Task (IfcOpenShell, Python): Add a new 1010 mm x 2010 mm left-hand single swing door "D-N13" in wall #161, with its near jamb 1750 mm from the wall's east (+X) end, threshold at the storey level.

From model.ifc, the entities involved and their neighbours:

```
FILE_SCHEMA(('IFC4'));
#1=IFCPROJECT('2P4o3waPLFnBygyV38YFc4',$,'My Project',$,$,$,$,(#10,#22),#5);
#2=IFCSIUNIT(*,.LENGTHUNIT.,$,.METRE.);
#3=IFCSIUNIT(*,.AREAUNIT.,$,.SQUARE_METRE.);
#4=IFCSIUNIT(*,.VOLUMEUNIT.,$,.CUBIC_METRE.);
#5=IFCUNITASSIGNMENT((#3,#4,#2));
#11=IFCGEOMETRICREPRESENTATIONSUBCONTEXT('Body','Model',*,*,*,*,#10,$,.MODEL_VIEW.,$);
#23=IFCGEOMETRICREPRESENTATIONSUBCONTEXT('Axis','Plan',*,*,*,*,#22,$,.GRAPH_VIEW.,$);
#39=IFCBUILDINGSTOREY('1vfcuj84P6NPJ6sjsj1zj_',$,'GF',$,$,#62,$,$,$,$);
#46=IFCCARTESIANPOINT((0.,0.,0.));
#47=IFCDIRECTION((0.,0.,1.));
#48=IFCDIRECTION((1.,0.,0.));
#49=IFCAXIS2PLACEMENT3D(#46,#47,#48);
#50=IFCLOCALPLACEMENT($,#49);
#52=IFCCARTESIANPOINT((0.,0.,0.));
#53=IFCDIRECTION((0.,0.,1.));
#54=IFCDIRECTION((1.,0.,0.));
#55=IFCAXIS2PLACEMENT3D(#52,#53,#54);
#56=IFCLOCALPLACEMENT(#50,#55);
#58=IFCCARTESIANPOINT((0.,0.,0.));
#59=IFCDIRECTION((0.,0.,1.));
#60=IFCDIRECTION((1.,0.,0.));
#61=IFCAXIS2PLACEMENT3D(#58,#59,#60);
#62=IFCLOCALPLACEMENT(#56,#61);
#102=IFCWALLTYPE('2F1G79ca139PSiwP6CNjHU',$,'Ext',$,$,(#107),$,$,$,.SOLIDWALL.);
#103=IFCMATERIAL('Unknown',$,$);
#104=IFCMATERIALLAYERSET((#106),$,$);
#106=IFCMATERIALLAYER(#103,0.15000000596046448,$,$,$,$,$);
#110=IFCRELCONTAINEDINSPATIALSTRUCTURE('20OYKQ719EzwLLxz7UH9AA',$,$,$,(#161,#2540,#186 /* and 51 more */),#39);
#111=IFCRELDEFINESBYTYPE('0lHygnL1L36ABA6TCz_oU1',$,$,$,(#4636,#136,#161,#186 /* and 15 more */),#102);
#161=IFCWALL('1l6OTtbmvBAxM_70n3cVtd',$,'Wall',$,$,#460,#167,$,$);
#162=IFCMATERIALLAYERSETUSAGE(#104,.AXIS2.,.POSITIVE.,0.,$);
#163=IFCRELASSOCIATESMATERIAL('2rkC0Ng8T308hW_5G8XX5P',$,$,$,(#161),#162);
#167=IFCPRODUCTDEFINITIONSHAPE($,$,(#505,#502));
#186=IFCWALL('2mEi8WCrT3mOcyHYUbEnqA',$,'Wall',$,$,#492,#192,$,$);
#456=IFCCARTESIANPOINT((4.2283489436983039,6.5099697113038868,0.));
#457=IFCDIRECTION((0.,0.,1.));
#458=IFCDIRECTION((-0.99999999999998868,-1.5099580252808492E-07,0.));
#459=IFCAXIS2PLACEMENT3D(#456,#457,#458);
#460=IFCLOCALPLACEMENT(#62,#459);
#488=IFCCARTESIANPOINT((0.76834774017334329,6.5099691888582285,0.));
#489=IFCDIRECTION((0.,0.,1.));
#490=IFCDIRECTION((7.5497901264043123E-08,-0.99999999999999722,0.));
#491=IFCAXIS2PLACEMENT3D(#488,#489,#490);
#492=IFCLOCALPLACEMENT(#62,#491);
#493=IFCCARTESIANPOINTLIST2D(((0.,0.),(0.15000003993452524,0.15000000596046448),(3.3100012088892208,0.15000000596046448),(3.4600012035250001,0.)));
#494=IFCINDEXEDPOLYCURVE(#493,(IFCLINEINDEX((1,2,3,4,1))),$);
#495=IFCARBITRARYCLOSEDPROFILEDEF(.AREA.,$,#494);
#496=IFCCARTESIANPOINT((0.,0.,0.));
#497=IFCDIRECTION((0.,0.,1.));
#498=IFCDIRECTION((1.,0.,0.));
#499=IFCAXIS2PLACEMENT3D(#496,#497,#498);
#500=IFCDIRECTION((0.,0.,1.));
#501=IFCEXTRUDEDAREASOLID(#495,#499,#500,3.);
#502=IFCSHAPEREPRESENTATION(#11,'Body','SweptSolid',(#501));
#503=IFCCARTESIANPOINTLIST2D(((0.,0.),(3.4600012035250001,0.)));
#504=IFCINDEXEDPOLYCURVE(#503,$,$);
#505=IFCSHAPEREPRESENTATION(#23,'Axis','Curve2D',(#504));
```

```python
import numpy as np
import ifcopenshell
import ifcopenshell.api.feature
import ifcopenshell.api.geometry
import ifcopenshell.api.root
import ifcopenshell.api.spatial
import ifcopenshell.geom
import ifcopenshell.util.element
import ifcopenshell.util.placement
import ifcopenshell.util.representation
import ifcopenshell.util.shape
import ifcopenshell.util.unit

model = ifcopenshell.open("model.ifc")
unit_scale = ifcopenshell.util.unit.calculate_unit_scale(model)
settings = ifcopenshell.geom.settings()


def volume(element):
    """Net volume in cubic metres, openings subtracted."""
    shape = ifcopenshell.geom.create_shape(settings, element)
    return ifcopenshell.util.shape.get_volume(shape.geometry)


wall = model.by_id(161)
storey = ifcopenshell.util.element.get_container(wall, ifc_class="IfcBuildingStorey")
context = ifcopenshell.util.representation.get_context(model, "Model", "Body", "MODEL_VIEW")
before = volume(wall)

width, height, from_end, sill = 1.01, 2.01, 1.75, 0.0  # metres

# The wall runs along its own X axis, and the end named is its -X end.
wall_shape = ifcopenshell.geom.create_shape(settings, wall)
x, y, z = ifcopenshell.util.shape.get_vertices(wall_shape.geometry).T
start = x.min() + from_end
face, thickness = float(y.min()), float(y.max() - y.min())
wall_matrix = ifcopenshell.util.placement.get_local_placement(wall.ObjectPlacement)
level = ifcopenshell.util.placement.get_local_placement(storey.ObjectPlacement)[2, 3]


def in_wall(x, y):
    """Placement at x, y metres in the wall's axes, at sill height."""
    matrix = wall_matrix.copy()
    matrix[:, 3] = wall_matrix @ np.array([x / unit_scale, y / unit_scale, 0.0, 1.0])
    matrix[2, 3] = level + sill / unit_scale
    return matrix


# Opening: a box that overshoots both wall faces by 50 mm.
opening = ifcopenshell.api.root.create_entity(model, ifc_class="IfcOpeningElement", predefined_type="OPENING")
box = ifcopenshell.api.geometry.add_wall_representation(
    model, context=context, length=width, height=height, thickness=thickness + 0.1
)
ifcopenshell.api.geometry.assign_representation(model, product=opening, representation=box)
ifcopenshell.api.geometry.edit_object_placement(model, product=opening, matrix=in_wall(start, face - 0.05), is_si=False)
ifcopenshell.api.feature.add_feature(model, feature=opening, element=wall)

door = ifcopenshell.api.root.create_entity(model, ifc_class="IfcDoor", name="D-N13", predefined_type="DOOR")
door.OverallWidth, door.OverallHeight = width / unit_scale, height / unit_scale
door.OperationType = "SINGLE_SWING_LEFT"
body = ifcopenshell.api.geometry.add_door_representation(
    model,
    context=context,
    overall_width=door.OverallWidth,
    overall_height=door.OverallHeight,
    operation_type="SINGLE_SWING_LEFT",
    lining_properties={"LiningDepth": thickness / unit_scale, "ThresholdDepth": thickness / unit_scale},
)
ifcopenshell.api.geometry.assign_representation(model, product=door, representation=body)
ifcopenshell.api.spatial.assign_container(model, products=[door], relating_structure=storey)
ifcopenshell.api.feature.add_filling(model, opening=opening, element=door)

# The lining spans the wall, so the door starts at the wall face.
ifcopenshell.api.geometry.edit_object_placement(model, product=door, matrix=in_wall(start, face), is_si=False)

after = volume(wall)

print(f"wall volume {before:.3f} -> {after:.3f} m3")

model.write("model_rev.ifc")
```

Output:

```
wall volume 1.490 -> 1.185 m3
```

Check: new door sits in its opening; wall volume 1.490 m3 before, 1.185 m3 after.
